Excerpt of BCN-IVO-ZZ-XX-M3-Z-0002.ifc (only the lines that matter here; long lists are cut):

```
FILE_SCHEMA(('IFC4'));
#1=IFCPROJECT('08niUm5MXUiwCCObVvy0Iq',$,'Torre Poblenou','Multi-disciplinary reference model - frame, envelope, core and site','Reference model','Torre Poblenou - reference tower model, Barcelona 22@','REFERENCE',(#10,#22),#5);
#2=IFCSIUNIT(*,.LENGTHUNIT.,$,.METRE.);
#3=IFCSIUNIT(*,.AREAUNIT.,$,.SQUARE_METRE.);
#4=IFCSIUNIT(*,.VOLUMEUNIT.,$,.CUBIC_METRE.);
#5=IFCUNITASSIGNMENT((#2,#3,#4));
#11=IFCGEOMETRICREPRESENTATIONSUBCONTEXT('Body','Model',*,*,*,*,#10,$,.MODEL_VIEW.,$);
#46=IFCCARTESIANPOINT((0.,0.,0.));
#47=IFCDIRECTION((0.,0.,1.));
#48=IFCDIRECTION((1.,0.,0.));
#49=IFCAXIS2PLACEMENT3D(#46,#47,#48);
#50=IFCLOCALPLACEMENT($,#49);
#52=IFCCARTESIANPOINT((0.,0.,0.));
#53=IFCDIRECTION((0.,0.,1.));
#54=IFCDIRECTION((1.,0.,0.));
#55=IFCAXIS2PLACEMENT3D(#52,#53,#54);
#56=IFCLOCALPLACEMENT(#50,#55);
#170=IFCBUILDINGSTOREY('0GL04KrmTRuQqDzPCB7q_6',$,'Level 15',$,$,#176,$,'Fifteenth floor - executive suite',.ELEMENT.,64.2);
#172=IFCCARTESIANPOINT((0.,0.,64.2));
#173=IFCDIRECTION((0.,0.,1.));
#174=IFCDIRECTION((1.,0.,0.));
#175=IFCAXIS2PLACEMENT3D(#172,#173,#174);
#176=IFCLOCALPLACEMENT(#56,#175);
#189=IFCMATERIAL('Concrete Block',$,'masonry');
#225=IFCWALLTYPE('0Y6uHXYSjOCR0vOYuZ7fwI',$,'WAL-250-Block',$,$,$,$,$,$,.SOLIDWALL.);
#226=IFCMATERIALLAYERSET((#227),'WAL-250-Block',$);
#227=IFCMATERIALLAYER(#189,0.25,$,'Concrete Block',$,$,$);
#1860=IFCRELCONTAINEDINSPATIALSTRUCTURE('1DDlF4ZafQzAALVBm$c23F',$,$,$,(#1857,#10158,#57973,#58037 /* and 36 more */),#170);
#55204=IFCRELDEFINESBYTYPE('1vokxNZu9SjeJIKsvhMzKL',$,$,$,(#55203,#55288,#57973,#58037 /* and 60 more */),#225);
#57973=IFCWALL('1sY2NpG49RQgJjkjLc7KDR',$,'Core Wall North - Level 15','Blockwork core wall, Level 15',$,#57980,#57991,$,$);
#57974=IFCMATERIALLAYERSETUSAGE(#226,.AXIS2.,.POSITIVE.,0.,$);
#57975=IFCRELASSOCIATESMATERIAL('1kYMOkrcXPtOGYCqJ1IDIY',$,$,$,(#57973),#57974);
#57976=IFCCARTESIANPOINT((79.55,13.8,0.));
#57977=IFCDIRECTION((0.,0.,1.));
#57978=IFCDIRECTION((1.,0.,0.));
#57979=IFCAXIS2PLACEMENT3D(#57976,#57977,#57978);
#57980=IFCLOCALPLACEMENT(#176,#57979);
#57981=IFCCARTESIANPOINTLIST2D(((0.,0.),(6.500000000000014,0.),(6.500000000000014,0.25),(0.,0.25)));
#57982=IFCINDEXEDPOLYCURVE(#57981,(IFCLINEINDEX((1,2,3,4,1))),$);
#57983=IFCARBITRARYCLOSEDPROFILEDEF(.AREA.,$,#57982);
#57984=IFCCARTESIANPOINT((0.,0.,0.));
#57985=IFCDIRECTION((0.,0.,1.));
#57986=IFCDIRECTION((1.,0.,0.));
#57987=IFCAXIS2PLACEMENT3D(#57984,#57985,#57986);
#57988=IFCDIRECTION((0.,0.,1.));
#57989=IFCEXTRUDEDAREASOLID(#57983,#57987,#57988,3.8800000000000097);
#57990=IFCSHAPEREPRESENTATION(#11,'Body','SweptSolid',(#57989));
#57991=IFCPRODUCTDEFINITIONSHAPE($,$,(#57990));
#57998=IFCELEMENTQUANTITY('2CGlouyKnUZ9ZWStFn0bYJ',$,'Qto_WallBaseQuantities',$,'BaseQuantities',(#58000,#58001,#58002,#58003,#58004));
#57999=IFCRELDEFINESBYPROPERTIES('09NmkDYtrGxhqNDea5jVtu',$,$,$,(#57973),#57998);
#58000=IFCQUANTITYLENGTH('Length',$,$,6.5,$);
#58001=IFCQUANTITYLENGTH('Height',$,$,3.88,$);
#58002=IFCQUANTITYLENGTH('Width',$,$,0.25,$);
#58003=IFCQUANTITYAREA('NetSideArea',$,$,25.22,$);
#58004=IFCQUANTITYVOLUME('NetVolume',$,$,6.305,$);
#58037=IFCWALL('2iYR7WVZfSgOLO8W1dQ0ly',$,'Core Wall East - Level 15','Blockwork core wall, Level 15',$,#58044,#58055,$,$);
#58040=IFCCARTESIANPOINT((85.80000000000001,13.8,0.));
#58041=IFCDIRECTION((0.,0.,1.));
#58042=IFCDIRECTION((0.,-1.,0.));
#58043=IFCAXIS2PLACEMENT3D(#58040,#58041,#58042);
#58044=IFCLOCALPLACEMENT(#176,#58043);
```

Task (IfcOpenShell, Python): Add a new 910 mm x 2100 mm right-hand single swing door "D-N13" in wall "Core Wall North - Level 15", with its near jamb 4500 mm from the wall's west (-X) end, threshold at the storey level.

```python
import numpy as np
import ifcopenshell
import ifcopenshell.api.feature
import ifcopenshell.api.geometry
import ifcopenshell.api.pset
import ifcopenshell.api.root
import ifcopenshell.api.spatial
import ifcopenshell.geom
import ifcopenshell.util.element
import ifcopenshell.util.placement
import ifcopenshell.util.representation
import ifcopenshell.util.shape
import ifcopenshell.util.unit

model = ifcopenshell.open("BCN-IVO-ZZ-XX-M3-Z-0002.ifc")
unit_scale = ifcopenshell.util.unit.calculate_unit_scale(model)
area_scale = ifcopenshell.util.unit.calculate_unit_scale(model, "AREAUNIT")
volume_scale = ifcopenshell.util.unit.calculate_unit_scale(model, "VOLUMEUNIT")
settings = ifcopenshell.geom.settings()


def volume(element):
    """Net volume in cubic metres, openings subtracted."""
    shape = ifcopenshell.geom.create_shape(settings, element)
    return ifcopenshell.util.shape.get_volume(shape.geometry)


wall = model.by_guid("1sY2NpG49RQgJjkjLc7KDR")
storey = ifcopenshell.util.element.get_container(wall, ifc_class="IfcBuildingStorey")
context = ifcopenshell.util.representation.get_context(model, "Model", "Body", "MODEL_VIEW")
before = volume(wall)

width, height, from_end, sill = 0.91, 2.1, 4.5, 0.0  # metres

# The wall runs along its own X axis, and the end named is its -X end.
wall_shape = ifcopenshell.geom.create_shape(settings, wall)
x, y, z = ifcopenshell.util.shape.get_vertices(wall_shape.geometry).T
start = x.min() + from_end
face, thickness = float(y.min()), float(y.max() - y.min())
wall_matrix = ifcopenshell.util.placement.get_local_placement(wall.ObjectPlacement)
level = ifcopenshell.util.placement.get_local_placement(storey.ObjectPlacement)[2, 3]


def in_wall(x, y):
    """Placement at x, y metres in the wall's axes, at sill height."""
    matrix = wall_matrix.copy()
    matrix[:, 3] = wall_matrix @ np.array([x / unit_scale, y / unit_scale, 0.0, 1.0])
    matrix[2, 3] = level + sill / unit_scale
    return matrix


# Opening: a box that overshoots both wall faces by 50 mm.
opening = ifcopenshell.api.root.create_entity(model, ifc_class="IfcOpeningElement", predefined_type="OPENING")
box = ifcopenshell.api.geometry.add_wall_representation(
    model, context=context, length=width, height=height, thickness=thickness + 0.1
)
ifcopenshell.api.geometry.assign_representation(model, product=opening, representation=box)
ifcopenshell.api.geometry.edit_object_placement(model, product=opening, matrix=in_wall(start, face - 0.05), is_si=False)
ifcopenshell.api.feature.add_feature(model, feature=opening, element=wall)

door = ifcopenshell.api.root.create_entity(model, ifc_class="IfcDoor", name="D-N13", predefined_type="DOOR")
door.OverallWidth, door.OverallHeight = width / unit_scale, height / unit_scale
door.OperationType = "SINGLE_SWING_RIGHT"
body = ifcopenshell.api.geometry.add_door_representation(
    model,
    context=context,
    overall_width=door.OverallWidth,
    overall_height=door.OverallHeight,
    operation_type="SINGLE_SWING_RIGHT",
    lining_properties={"LiningDepth": thickness / unit_scale, "ThresholdDepth": thickness / unit_scale},
)
ifcopenshell.api.geometry.assign_representation(model, product=door, representation=body)
ifcopenshell.api.spatial.assign_container(model, products=[door], relating_structure=storey)
ifcopenshell.api.feature.add_filling(model, opening=opening, element=door)

# The lining spans the wall, so the door starts at the wall face.
ifcopenshell.api.geometry.edit_object_placement(model, product=door, matrix=in_wall(start, face), is_si=False)

after = volume(wall)

# Update the wall's stored quantities.
qto = model.by_id(ifcopenshell.util.element.get_pset(wall, "Qto_WallBaseQuantities", should_inherit=False)["id"])
ifcopenshell.api.pset.edit_qto(model, qto=qto, properties={
    "NetSideArea": after / thickness / area_scale,
    "NetVolume": after / volume_scale,
})

print(f"wall volume {before:.3f} -> {after:.3f} m3")

model.write("BCN-IVO-ZZ-XX-M3-Z-0002_updated.ifc")
```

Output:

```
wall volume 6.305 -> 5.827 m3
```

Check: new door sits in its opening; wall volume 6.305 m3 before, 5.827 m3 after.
